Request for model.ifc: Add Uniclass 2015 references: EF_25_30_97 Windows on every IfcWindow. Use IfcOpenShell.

First a look at what the model holds.

```python
import ifcopenshell

model = ifcopenshell.open("model.ifc")
print(model.schema)
print("classifications:", [c.Name for c in model.by_type("IfcClassification")])
for ifc_class in ("IfcDoor", "IfcRoof", "IfcStair", "IfcWall", "IfcWindow"):
    print(ifc_class, len(model.by_type(ifc_class)))
```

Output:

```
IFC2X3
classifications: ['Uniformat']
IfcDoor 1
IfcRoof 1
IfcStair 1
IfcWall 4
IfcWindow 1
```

```python
import ifcopenshell
import ifcopenshell.api.classification

model = ifcopenshell.open("model.ifc")

# IFC2X3 requires Source and Edition and has no link from the project to the system.
system = model.create_entity("IfcClassification", Source="NBS", Edition="2015", Name="Uniclass 2015")

codes = {
    "IfcWindow": ("EF_25_30_97", "Windows"),
}
for ifc_class, (code, name) in codes.items():
    products = model.by_type(ifc_class)
    ifcopenshell.api.classification.add_reference(
        model, products=products, classification=system, identification=code, name=name
    )
    print(code, len(products))

model.write("model_rev.ifc")
```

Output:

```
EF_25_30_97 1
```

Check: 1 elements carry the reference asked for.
